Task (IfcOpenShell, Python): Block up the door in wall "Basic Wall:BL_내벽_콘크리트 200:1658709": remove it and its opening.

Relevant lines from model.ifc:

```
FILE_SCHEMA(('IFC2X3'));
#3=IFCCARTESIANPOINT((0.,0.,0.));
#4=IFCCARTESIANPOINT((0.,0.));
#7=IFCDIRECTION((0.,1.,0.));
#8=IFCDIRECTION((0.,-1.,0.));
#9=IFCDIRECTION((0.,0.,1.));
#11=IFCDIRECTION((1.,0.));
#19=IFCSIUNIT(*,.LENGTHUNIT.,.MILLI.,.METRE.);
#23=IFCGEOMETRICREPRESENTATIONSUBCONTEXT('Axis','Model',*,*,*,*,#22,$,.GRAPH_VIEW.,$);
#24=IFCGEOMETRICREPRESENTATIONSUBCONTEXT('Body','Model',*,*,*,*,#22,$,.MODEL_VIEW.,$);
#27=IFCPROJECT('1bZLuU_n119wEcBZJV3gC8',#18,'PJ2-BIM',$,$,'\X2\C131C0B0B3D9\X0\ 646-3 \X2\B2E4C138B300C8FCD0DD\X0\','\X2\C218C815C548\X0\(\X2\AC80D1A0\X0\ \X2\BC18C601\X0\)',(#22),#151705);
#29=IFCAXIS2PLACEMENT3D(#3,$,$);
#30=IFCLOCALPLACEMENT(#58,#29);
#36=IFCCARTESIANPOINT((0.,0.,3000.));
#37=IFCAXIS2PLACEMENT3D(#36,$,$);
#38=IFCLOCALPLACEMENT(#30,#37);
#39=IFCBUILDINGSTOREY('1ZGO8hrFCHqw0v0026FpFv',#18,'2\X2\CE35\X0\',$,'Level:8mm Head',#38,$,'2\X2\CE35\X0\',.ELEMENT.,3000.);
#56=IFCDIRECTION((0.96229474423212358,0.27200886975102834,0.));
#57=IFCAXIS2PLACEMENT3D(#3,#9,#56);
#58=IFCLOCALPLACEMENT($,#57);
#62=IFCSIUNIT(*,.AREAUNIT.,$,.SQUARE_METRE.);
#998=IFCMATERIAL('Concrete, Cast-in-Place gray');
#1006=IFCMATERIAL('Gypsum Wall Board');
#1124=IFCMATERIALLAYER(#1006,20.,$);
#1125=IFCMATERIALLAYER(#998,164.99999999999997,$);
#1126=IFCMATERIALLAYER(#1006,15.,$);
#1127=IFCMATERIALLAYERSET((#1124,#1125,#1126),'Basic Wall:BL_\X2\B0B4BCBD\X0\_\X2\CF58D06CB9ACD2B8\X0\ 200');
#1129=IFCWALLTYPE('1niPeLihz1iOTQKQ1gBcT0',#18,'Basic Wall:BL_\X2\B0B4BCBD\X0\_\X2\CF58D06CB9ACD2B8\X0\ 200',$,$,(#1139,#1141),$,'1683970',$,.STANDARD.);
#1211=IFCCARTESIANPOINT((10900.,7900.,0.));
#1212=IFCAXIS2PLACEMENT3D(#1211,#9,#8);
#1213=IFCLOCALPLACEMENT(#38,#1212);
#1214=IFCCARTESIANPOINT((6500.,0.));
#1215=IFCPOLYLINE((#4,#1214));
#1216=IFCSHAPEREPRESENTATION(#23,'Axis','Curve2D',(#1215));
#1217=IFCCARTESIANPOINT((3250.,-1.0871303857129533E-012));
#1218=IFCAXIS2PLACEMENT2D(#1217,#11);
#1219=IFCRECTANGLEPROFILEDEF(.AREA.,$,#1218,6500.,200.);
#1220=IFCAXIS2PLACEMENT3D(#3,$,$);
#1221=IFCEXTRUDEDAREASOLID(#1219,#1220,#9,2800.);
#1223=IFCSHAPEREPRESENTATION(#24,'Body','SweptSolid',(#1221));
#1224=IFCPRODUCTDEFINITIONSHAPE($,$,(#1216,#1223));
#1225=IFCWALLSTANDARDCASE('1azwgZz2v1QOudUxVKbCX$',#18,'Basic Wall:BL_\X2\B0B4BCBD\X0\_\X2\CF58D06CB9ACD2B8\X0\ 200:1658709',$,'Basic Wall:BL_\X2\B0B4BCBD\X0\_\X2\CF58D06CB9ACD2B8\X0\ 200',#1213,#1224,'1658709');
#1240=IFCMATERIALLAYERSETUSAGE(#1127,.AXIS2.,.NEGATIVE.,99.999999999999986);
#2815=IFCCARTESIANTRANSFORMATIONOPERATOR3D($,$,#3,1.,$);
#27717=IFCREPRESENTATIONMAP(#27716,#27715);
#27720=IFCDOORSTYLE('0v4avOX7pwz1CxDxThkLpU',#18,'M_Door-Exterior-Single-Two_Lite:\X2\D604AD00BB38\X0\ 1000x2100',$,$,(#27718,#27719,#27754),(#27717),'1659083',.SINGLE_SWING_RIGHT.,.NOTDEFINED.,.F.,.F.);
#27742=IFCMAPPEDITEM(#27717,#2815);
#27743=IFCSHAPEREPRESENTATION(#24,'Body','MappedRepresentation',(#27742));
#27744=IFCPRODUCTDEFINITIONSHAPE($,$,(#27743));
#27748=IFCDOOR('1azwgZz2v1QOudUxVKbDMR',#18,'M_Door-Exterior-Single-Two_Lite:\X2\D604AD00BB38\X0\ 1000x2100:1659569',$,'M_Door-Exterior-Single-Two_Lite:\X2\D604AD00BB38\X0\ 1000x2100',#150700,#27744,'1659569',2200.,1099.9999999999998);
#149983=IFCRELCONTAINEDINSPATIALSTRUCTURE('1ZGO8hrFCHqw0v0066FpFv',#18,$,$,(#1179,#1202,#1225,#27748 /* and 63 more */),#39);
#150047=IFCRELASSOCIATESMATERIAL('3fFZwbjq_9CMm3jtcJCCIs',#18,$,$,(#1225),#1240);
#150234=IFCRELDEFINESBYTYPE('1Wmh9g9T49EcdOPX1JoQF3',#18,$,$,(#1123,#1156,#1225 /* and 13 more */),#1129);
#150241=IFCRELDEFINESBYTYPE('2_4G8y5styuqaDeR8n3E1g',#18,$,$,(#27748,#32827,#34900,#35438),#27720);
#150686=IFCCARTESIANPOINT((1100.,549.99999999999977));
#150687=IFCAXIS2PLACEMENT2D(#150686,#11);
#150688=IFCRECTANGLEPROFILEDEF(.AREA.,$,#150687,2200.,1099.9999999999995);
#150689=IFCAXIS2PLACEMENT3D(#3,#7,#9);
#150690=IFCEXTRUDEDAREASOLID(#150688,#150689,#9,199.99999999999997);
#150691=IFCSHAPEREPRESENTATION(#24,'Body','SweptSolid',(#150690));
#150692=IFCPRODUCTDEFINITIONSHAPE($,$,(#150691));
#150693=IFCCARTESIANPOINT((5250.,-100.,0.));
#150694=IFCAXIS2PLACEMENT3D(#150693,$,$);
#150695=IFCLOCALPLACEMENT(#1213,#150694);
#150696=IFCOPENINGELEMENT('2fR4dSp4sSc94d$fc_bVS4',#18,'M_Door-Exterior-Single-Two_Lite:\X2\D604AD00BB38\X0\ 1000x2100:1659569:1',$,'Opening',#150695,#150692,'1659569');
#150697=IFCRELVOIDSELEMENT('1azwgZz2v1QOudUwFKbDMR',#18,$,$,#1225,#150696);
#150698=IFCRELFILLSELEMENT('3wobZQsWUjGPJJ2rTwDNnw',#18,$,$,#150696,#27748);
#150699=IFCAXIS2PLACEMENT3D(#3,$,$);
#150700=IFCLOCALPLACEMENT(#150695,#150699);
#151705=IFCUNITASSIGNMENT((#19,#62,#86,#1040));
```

```python
import ifcopenshell
import ifcopenshell.api.feature
import ifcopenshell.api.root
import ifcopenshell.geom
import ifcopenshell.util.shape

model = ifcopenshell.open("model.ifc")
settings = ifcopenshell.geom.settings()


def volume(element):
    """Net volume in cubic metres, openings subtracted."""
    shape = ifcopenshell.geom.create_shape(settings, element)
    return ifcopenshell.util.shape.get_volume(shape.geometry)


door = model.by_guid("1azwgZz2v1QOudUxVKbDMR")
opening = door.FillsVoids[0].RelatingOpeningElement
wall = opening.VoidsElements[0].RelatingBuildingElement
before = volume(wall)

ifcopenshell.api.root.remove_product(model, product=door)
ifcopenshell.api.feature.remove_feature(model, feature=opening)

after = volume(wall)

print(f"wall volume {before:.3f} -> {after:.3f} m3")

model.write("model_edited.ifc")
```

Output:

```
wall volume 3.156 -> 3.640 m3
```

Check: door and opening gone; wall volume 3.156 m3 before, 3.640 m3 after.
